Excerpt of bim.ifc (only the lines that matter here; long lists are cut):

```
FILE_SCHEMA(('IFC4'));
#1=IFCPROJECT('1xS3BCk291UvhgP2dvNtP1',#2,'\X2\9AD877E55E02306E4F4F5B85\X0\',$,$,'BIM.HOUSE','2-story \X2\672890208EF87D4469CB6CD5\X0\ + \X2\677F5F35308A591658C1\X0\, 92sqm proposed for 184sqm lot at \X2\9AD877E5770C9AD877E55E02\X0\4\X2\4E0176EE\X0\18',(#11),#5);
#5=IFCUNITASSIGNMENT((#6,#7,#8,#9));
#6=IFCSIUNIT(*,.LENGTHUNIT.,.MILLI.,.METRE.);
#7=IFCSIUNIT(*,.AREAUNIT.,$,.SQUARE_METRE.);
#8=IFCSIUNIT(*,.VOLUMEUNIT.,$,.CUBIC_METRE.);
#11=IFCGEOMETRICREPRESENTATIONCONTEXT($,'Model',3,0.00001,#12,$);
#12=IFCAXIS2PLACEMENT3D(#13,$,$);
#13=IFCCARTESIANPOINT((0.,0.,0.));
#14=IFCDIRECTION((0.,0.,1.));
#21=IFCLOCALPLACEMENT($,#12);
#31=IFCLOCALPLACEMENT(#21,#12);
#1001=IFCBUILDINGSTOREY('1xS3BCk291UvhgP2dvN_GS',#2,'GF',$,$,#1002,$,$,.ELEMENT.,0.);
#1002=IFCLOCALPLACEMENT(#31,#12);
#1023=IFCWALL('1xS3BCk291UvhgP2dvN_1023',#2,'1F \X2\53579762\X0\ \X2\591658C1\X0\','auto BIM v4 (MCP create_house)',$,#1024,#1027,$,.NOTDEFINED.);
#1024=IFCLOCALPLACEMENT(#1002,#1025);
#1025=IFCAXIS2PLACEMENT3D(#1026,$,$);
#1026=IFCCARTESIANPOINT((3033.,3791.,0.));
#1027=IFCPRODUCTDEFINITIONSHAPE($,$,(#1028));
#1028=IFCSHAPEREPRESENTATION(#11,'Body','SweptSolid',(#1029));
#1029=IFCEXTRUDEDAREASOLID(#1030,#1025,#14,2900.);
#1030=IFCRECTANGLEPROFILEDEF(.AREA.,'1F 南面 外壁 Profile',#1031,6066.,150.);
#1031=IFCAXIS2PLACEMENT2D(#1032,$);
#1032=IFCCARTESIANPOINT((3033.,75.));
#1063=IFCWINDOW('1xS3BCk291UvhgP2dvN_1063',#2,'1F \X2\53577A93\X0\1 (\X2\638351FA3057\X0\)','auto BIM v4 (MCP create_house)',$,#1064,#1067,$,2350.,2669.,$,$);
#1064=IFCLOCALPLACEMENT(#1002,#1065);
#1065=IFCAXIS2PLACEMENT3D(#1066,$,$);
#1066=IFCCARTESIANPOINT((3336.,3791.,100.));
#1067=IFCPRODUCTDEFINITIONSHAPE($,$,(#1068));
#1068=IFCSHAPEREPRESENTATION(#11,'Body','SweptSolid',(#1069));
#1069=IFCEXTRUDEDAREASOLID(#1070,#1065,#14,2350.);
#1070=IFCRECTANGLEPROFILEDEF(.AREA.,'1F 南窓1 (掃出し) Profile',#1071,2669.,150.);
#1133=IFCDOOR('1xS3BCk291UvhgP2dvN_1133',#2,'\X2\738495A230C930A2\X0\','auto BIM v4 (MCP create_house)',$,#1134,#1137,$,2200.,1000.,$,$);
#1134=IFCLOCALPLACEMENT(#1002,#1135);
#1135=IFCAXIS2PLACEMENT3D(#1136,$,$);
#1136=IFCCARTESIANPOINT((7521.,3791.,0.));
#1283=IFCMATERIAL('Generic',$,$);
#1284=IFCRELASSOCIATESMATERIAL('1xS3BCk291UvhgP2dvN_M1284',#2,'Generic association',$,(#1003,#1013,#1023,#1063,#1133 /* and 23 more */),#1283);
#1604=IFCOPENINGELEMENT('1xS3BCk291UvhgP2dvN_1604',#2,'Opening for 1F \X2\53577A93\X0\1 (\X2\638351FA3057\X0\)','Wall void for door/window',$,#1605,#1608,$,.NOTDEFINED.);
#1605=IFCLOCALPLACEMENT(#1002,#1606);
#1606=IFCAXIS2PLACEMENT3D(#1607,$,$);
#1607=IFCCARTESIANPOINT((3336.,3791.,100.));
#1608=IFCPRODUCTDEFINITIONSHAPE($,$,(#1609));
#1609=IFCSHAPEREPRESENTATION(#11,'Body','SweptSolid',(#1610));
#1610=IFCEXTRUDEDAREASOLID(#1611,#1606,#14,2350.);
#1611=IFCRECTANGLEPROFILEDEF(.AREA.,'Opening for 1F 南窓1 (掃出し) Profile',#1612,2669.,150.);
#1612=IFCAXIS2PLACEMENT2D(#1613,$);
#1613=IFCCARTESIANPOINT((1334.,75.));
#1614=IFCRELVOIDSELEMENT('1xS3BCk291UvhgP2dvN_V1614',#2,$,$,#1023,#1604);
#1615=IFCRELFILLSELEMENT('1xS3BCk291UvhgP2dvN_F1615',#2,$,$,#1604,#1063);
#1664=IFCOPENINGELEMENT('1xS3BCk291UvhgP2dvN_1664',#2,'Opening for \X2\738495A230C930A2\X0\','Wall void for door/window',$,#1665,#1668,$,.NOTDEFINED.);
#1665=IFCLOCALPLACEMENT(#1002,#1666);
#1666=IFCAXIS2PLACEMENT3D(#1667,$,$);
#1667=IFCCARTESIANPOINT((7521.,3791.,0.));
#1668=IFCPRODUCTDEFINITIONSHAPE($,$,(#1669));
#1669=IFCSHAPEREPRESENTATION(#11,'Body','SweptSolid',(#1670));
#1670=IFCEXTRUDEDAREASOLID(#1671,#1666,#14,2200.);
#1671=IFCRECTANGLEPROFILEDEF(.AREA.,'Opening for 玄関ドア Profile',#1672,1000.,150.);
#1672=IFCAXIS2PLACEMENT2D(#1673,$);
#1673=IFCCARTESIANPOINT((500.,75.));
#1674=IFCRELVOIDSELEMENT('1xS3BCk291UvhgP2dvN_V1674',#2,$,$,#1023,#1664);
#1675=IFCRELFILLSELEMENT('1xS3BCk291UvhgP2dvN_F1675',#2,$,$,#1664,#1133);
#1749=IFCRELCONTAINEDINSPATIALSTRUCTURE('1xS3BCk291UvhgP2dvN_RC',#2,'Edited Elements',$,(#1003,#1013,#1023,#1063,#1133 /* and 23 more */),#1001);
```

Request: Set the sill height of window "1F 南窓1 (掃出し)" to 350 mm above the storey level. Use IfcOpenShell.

```python
import numpy as np
import ifcopenshell
import ifcopenshell.api.geometry
import ifcopenshell.geom
import ifcopenshell.util.element
import ifcopenshell.util.placement
import ifcopenshell.util.shape
import ifcopenshell.util.unit

model = ifcopenshell.open("bim.ifc")
unit_scale = ifcopenshell.util.unit.calculate_unit_scale(model)

window = model.by_guid("1xS3BCk291UvhgP2dvN_1063")
opening = window.FillsVoids[0].RelatingOpeningElement
storey = ifcopenshell.util.element.get_container(window, ifc_class="IfcBuildingStorey")
level = ifcopenshell.util.placement.get_local_placement(storey.ObjectPlacement)[2, 3]

# The opening's origin need not be at the sill, so measure its lowest point.
shape = ifcopenshell.geom.create_shape(ifcopenshell.geom.settings(), opening)
bottom = ifcopenshell.util.shape.get_shape_bottom_elevation(shape, shape.geometry) / unit_scale
dz = level + 350.0 - bottom

shift = np.array([0.0, 0.0, dz])
# The window is not placed relative to its opening, so move both.
for product in (opening, window):
    matrix = ifcopenshell.util.placement.get_local_placement(product.ObjectPlacement)
    matrix[:3, 3] += shift
    ifcopenshell.api.geometry.edit_object_placement(model, product=product, matrix=matrix, is_si=False)

print(f"moved by {dz * unit_scale:+.3f} m")

model.write("bim-out.ifc")
```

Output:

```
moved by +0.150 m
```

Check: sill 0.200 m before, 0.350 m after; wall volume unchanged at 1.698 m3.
